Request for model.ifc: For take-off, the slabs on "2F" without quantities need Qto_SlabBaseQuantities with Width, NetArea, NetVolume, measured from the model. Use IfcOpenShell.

First a look at what the model holds.

```python
import ifcopenshell
import ifcopenshell.util.element
import ifcopenshell.util.unit

model = ifcopenshell.open("model.ifc")
print(model.schema)
for unit_type in ("LENGTHUNIT", "AREAUNIT", "VOLUMEUNIT"):
    print(unit_type, ifcopenshell.util.unit.calculate_unit_scale(model, unit_type))
storey = next(s for s in model.by_type("IfcBuildingStorey") if s.Name == "2F")
slabs = [e for e in ifcopenshell.util.element.get_decomposition(storey) if e.is_a("IfcSlab")]
for e in sorted(slabs, key=lambda e: e.id()):
    print(e.id(), e.is_a(), e.Name, list(ifcopenshell.util.element.get_psets(e, qtos_only=True)), sep=" | ")
```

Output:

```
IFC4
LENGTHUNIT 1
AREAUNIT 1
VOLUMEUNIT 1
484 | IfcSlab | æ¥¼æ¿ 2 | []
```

```python
import ifcopenshell
import ifcopenshell.api.pset
import ifcopenshell.geom
import ifcopenshell.util.element
import ifcopenshell.util.shape
import ifcopenshell.util.unit

model = ifcopenshell.open("model.ifc")
unit_scale = ifcopenshell.util.unit.calculate_unit_scale(model)
area_scale = ifcopenshell.util.unit.calculate_unit_scale(model, "AREAUNIT")
volume_scale = ifcopenshell.util.unit.calculate_unit_scale(model, "VOLUMEUNIT")
settings = ifcopenshell.geom.settings()

storey = next(s for s in model.by_type("IfcBuildingStorey") if s.Name == "2F")
slabs = [e for e in ifcopenshell.util.element.get_decomposition(storey) if e.is_a("IfcSlab")]

for e in sorted(slabs, key=lambda e: e.id()):
    if ifcopenshell.util.element.get_psets(e, qtos_only=True, should_inherit=False):
        continue
    # Geometry comes back in metres, in the element's own axes.
    shape = ifcopenshell.geom.create_shape(settings, e)
    values = {
        "Width": ifcopenshell.util.shape.get_z(shape.geometry) / unit_scale,
        "NetArea": ifcopenshell.util.shape.get_footprint_area(shape.geometry) / area_scale,
        "NetVolume": ifcopenshell.util.shape.get_volume(shape.geometry) / volume_scale,
    }
    qto = ifcopenshell.api.pset.add_qto(model, product=e, name="Qto_SlabBaseQuantities")
    ifcopenshell.api.pset.edit_qto(model, qto=qto, properties=values)
    print(e.id(), {k: round(v, 3) for k, v in values.items()})

model.write("model_v2.ifc")
```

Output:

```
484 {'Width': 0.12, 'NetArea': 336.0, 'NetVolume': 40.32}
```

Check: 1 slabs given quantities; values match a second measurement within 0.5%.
